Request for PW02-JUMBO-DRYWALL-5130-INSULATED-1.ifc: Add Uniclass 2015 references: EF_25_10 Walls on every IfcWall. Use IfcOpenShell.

First a look at what the model holds.

```python
import ifcopenshell

model = ifcopenshell.open("PW02-JUMBO-DRYWALL-5130-INSULATED-1.ifc")
print(model.schema)
print("classifications:", [c.Name for c in model.by_type("IfcClassification")])
for ifc_class in ("IfcDoor", "IfcRoof", "IfcStair", "IfcWall", "IfcWindow"):
    print(ifc_class, len(model.by_type(ifc_class)))
```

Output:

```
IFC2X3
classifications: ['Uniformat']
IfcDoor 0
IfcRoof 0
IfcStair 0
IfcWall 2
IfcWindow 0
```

```python
import ifcopenshell
import ifcopenshell.api.classification

model = ifcopenshell.open("PW02-JUMBO-DRYWALL-5130-INSULATED-1.ifc")

# IFC2X3 requires Source and Edition and has no link from the project to the system.
system = model.create_entity("IfcClassification", Source="NBS", Edition="2015", Name="Uniclass 2015")

codes = {
    "IfcWall": ("EF_25_10", "Walls"),
}
for ifc_class, (code, name) in codes.items():
    products = model.by_type(ifc_class)
    ifcopenshell.api.classification.add_reference(
        model, products=products, classification=system, identification=code, name=name
    )
    print(code, len(products))

model.write("PW02-JUMBO-DRYWALL-5130-INSULATED-1_v2.ifc")
```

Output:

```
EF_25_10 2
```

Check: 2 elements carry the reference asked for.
